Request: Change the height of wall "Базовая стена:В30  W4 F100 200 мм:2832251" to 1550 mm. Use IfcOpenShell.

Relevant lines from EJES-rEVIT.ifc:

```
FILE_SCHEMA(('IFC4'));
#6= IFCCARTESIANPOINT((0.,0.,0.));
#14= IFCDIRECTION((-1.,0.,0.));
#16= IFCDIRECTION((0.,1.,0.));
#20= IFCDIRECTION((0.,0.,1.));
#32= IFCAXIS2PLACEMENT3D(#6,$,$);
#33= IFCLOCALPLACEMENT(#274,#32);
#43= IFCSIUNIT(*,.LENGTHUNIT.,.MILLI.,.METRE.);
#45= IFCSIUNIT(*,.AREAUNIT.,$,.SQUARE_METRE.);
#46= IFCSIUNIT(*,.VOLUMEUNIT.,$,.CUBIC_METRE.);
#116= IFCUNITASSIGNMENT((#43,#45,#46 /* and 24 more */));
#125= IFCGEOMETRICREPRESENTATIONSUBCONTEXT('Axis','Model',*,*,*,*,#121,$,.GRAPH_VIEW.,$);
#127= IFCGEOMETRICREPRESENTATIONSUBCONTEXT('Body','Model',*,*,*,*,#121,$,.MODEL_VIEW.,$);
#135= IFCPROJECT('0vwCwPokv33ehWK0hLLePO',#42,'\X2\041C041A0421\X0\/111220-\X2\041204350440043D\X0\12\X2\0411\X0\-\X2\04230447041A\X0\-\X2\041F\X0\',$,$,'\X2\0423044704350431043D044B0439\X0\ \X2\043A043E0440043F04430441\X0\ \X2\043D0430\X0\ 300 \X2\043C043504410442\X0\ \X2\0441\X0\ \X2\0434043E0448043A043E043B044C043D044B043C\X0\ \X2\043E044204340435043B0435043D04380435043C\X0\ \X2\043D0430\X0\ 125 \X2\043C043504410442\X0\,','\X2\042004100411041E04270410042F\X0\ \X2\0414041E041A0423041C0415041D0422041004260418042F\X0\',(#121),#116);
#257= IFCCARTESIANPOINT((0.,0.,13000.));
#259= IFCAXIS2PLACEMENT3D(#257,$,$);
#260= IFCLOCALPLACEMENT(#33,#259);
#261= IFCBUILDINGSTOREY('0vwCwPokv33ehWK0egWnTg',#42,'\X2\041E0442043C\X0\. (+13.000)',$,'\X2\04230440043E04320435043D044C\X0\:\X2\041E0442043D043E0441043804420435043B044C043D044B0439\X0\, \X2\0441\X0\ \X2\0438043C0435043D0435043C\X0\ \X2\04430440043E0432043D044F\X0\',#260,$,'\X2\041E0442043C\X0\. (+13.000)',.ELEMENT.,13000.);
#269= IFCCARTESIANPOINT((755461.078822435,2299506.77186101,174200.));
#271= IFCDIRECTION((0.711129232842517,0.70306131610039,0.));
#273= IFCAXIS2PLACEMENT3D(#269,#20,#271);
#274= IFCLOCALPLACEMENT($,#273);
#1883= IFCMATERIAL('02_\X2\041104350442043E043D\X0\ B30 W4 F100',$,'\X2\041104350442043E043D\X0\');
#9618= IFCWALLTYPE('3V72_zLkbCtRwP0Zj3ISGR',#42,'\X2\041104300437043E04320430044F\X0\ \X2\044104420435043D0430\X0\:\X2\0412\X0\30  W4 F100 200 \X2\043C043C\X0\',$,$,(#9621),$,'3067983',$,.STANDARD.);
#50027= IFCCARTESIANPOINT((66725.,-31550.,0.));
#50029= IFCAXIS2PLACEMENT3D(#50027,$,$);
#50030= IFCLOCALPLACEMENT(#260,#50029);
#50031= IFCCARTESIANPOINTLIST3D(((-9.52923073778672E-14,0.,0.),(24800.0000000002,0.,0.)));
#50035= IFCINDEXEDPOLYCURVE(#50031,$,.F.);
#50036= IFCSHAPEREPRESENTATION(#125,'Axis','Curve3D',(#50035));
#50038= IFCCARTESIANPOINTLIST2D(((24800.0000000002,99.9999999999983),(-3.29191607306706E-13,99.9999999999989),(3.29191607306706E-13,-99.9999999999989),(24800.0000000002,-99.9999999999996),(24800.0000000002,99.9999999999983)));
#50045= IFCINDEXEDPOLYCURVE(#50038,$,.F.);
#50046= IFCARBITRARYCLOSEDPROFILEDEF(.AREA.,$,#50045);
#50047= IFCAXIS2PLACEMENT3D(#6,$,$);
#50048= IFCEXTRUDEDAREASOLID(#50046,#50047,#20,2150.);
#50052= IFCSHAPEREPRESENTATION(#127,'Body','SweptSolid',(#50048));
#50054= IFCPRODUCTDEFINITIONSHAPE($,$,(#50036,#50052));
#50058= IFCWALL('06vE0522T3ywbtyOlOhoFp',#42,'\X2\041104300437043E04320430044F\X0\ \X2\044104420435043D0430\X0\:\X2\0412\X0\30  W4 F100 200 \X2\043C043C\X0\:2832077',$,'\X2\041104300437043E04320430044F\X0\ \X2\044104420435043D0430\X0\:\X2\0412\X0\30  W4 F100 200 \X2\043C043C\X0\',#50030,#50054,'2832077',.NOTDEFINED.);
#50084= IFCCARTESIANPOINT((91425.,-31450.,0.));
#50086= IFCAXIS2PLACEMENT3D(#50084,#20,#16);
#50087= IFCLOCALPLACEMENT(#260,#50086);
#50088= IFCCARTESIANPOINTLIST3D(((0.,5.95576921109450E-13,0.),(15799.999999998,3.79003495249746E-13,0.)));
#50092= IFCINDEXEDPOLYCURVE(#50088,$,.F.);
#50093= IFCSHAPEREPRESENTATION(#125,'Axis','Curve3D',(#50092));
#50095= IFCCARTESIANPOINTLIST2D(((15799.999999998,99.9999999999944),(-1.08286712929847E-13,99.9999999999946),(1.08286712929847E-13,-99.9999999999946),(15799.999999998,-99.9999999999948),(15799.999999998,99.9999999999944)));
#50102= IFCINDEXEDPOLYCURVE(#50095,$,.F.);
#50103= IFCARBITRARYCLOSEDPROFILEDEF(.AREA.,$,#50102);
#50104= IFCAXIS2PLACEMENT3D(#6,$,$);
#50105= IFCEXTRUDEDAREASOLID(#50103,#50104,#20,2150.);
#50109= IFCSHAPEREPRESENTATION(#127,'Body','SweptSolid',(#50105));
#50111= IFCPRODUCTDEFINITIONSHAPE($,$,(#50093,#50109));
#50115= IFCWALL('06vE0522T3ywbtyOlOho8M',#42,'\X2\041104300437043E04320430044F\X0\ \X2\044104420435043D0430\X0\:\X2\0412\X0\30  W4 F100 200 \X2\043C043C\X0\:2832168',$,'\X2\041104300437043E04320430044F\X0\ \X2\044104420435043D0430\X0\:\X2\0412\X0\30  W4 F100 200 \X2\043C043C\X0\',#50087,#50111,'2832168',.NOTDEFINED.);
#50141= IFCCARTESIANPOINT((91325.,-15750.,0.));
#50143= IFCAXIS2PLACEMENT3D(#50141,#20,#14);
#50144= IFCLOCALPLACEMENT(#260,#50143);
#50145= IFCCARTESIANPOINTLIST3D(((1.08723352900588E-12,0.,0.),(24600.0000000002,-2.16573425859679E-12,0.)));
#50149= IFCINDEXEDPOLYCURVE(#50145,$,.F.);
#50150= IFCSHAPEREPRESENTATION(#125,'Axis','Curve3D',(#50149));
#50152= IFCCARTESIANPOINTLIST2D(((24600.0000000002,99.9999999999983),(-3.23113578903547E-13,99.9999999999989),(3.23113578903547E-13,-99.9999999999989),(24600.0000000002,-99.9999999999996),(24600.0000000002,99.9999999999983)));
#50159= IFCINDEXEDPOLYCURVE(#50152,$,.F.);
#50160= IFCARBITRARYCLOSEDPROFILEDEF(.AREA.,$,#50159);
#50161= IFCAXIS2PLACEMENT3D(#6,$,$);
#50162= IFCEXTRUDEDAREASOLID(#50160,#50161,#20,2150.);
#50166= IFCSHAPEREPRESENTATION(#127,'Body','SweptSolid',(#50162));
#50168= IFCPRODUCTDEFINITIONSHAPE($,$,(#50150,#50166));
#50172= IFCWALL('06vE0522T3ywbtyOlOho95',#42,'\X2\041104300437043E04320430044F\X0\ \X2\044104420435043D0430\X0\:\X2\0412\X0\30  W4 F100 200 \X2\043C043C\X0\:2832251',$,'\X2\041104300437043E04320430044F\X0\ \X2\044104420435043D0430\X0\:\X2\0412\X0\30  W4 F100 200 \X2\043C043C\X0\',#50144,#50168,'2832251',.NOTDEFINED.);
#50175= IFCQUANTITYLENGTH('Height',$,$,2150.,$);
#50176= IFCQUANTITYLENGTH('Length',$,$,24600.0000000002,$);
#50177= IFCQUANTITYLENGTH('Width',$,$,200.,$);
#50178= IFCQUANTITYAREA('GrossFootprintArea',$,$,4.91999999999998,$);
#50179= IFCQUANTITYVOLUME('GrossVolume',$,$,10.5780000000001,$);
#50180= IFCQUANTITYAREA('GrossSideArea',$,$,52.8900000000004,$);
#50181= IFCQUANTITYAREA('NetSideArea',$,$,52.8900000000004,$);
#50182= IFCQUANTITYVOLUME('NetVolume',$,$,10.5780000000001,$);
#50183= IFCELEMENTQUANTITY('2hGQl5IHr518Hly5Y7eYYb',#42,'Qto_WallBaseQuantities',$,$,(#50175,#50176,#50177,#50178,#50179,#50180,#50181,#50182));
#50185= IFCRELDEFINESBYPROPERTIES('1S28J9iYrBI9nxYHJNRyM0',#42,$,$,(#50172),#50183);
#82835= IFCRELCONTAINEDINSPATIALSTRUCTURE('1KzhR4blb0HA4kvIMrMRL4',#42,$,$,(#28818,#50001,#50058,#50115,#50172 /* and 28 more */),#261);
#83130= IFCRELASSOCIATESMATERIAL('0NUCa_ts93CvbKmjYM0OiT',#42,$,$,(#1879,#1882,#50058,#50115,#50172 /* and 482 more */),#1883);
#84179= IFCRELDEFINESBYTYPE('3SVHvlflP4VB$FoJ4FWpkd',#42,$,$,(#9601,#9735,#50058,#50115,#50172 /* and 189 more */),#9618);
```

```python
import ifcopenshell
import ifcopenshell.api.pset
import ifcopenshell.geom
import ifcopenshell.util.element
import ifcopenshell.util.representation
import ifcopenshell.util.shape
import ifcopenshell.util.unit

model = ifcopenshell.open("EJES-rEVIT.ifc")
unit_scale = ifcopenshell.util.unit.calculate_unit_scale(model)
area_scale = ifcopenshell.util.unit.calculate_unit_scale(model, "AREAUNIT")
volume_scale = ifcopenshell.util.unit.calculate_unit_scale(model, "VOLUMEUNIT")
settings = ifcopenshell.geom.settings()


def volume(element):
    """Net volume in cubic metres, openings subtracted."""
    shape = ifcopenshell.geom.create_shape(settings, element)
    return ifcopenshell.util.shape.get_volume(shape.geometry)


wall = model.by_id(50172)
before = volume(wall)

body = ifcopenshell.util.representation.get_representation(wall, "Model", "Body")
solid = body.Items[0]
old_height = solid.Depth
solid.Depth = 1550.0
after = volume(wall)
thickness = 0.2  # wall thickness in metres

# Update the stored height, areas and volumes.
qto = model.by_id(ifcopenshell.util.element.get_pset(wall, "Qto_WallBaseQuantities", should_inherit=False)["id"])
ifcopenshell.api.pset.edit_qto(model, qto=qto, properties={
    "Height": solid.Depth,
    "GrossVolume": ifcopenshell.util.element.get_pset(wall, "Qto_WallBaseQuantities", "GrossVolume") * solid.Depth / old_height,
    "GrossSideArea": ifcopenshell.util.element.get_pset(wall, "Qto_WallBaseQuantities", "GrossSideArea") * solid.Depth / old_height,
    "NetSideArea": after / thickness / area_scale,
    "NetVolume": after / volume_scale,
})

print(f"height {old_height:g} -> {solid.Depth:g}, volume {before:.3f} -> {after:.3f} m3")

model.write("EJES-rEVIT_v2.ifc")
```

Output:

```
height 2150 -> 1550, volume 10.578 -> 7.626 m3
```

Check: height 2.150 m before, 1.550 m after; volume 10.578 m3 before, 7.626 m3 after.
